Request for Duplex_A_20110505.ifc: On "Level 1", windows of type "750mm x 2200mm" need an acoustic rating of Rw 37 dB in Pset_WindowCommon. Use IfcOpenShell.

First a look at what the model holds.

```python
import ifcopenshell
import ifcopenshell.util.element

model = ifcopenshell.open("Duplex_A_20110505.ifc")
print(model.schema)
storey = next(s for s in model.by_type("IfcBuildingStorey") if s.Name == "Level 1")
windows = [e for e in ifcopenshell.util.element.get_decomposition(storey) if e.is_a("IfcWindow")]
seen = {}
for e in windows:
    element_type = ifcopenshell.util.element.get_type(e)
    key = (element_type.Name if element_type != e and element_type else None, ifcopenshell.util.element.get_pset(e, "Pset_WindowCommon", "AcousticRating"))
    seen[key] = seen.get(key, 0) + 1
for (name, value), count in sorted(seen.items(), key=str):
    print(count, "x", name, "|", value)
```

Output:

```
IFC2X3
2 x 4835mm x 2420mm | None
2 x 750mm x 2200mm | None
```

```python
import ifcopenshell
import ifcopenshell.api.pset
import ifcopenshell.util.element

model = ifcopenshell.open("Duplex_A_20110505.ifc")

storey = next(s for s in model.by_type("IfcBuildingStorey") if s.Name == "Level 1")
windows = [e for e in ifcopenshell.util.element.get_decomposition(storey) if e.is_a("IfcWindow")]

count = 0
for e in windows:
    element_type = ifcopenshell.util.element.get_type(e)
    if element_type in (None, e) or element_type.Name != "750mm x 2200mm":
        continue
    # add_pset returns the element's existing set when there is one.
    pset = ifcopenshell.api.pset.add_pset(model, product=e, name="Pset_WindowCommon")
    ifcopenshell.api.pset.edit_pset(model, pset=pset, properties={"AcousticRating": "Rw 37 dB"})
    count += 1

print(count, "windows updated")

model.write("Duplex_A_20110505_updated.ifc")
```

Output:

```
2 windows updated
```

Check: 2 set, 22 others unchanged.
